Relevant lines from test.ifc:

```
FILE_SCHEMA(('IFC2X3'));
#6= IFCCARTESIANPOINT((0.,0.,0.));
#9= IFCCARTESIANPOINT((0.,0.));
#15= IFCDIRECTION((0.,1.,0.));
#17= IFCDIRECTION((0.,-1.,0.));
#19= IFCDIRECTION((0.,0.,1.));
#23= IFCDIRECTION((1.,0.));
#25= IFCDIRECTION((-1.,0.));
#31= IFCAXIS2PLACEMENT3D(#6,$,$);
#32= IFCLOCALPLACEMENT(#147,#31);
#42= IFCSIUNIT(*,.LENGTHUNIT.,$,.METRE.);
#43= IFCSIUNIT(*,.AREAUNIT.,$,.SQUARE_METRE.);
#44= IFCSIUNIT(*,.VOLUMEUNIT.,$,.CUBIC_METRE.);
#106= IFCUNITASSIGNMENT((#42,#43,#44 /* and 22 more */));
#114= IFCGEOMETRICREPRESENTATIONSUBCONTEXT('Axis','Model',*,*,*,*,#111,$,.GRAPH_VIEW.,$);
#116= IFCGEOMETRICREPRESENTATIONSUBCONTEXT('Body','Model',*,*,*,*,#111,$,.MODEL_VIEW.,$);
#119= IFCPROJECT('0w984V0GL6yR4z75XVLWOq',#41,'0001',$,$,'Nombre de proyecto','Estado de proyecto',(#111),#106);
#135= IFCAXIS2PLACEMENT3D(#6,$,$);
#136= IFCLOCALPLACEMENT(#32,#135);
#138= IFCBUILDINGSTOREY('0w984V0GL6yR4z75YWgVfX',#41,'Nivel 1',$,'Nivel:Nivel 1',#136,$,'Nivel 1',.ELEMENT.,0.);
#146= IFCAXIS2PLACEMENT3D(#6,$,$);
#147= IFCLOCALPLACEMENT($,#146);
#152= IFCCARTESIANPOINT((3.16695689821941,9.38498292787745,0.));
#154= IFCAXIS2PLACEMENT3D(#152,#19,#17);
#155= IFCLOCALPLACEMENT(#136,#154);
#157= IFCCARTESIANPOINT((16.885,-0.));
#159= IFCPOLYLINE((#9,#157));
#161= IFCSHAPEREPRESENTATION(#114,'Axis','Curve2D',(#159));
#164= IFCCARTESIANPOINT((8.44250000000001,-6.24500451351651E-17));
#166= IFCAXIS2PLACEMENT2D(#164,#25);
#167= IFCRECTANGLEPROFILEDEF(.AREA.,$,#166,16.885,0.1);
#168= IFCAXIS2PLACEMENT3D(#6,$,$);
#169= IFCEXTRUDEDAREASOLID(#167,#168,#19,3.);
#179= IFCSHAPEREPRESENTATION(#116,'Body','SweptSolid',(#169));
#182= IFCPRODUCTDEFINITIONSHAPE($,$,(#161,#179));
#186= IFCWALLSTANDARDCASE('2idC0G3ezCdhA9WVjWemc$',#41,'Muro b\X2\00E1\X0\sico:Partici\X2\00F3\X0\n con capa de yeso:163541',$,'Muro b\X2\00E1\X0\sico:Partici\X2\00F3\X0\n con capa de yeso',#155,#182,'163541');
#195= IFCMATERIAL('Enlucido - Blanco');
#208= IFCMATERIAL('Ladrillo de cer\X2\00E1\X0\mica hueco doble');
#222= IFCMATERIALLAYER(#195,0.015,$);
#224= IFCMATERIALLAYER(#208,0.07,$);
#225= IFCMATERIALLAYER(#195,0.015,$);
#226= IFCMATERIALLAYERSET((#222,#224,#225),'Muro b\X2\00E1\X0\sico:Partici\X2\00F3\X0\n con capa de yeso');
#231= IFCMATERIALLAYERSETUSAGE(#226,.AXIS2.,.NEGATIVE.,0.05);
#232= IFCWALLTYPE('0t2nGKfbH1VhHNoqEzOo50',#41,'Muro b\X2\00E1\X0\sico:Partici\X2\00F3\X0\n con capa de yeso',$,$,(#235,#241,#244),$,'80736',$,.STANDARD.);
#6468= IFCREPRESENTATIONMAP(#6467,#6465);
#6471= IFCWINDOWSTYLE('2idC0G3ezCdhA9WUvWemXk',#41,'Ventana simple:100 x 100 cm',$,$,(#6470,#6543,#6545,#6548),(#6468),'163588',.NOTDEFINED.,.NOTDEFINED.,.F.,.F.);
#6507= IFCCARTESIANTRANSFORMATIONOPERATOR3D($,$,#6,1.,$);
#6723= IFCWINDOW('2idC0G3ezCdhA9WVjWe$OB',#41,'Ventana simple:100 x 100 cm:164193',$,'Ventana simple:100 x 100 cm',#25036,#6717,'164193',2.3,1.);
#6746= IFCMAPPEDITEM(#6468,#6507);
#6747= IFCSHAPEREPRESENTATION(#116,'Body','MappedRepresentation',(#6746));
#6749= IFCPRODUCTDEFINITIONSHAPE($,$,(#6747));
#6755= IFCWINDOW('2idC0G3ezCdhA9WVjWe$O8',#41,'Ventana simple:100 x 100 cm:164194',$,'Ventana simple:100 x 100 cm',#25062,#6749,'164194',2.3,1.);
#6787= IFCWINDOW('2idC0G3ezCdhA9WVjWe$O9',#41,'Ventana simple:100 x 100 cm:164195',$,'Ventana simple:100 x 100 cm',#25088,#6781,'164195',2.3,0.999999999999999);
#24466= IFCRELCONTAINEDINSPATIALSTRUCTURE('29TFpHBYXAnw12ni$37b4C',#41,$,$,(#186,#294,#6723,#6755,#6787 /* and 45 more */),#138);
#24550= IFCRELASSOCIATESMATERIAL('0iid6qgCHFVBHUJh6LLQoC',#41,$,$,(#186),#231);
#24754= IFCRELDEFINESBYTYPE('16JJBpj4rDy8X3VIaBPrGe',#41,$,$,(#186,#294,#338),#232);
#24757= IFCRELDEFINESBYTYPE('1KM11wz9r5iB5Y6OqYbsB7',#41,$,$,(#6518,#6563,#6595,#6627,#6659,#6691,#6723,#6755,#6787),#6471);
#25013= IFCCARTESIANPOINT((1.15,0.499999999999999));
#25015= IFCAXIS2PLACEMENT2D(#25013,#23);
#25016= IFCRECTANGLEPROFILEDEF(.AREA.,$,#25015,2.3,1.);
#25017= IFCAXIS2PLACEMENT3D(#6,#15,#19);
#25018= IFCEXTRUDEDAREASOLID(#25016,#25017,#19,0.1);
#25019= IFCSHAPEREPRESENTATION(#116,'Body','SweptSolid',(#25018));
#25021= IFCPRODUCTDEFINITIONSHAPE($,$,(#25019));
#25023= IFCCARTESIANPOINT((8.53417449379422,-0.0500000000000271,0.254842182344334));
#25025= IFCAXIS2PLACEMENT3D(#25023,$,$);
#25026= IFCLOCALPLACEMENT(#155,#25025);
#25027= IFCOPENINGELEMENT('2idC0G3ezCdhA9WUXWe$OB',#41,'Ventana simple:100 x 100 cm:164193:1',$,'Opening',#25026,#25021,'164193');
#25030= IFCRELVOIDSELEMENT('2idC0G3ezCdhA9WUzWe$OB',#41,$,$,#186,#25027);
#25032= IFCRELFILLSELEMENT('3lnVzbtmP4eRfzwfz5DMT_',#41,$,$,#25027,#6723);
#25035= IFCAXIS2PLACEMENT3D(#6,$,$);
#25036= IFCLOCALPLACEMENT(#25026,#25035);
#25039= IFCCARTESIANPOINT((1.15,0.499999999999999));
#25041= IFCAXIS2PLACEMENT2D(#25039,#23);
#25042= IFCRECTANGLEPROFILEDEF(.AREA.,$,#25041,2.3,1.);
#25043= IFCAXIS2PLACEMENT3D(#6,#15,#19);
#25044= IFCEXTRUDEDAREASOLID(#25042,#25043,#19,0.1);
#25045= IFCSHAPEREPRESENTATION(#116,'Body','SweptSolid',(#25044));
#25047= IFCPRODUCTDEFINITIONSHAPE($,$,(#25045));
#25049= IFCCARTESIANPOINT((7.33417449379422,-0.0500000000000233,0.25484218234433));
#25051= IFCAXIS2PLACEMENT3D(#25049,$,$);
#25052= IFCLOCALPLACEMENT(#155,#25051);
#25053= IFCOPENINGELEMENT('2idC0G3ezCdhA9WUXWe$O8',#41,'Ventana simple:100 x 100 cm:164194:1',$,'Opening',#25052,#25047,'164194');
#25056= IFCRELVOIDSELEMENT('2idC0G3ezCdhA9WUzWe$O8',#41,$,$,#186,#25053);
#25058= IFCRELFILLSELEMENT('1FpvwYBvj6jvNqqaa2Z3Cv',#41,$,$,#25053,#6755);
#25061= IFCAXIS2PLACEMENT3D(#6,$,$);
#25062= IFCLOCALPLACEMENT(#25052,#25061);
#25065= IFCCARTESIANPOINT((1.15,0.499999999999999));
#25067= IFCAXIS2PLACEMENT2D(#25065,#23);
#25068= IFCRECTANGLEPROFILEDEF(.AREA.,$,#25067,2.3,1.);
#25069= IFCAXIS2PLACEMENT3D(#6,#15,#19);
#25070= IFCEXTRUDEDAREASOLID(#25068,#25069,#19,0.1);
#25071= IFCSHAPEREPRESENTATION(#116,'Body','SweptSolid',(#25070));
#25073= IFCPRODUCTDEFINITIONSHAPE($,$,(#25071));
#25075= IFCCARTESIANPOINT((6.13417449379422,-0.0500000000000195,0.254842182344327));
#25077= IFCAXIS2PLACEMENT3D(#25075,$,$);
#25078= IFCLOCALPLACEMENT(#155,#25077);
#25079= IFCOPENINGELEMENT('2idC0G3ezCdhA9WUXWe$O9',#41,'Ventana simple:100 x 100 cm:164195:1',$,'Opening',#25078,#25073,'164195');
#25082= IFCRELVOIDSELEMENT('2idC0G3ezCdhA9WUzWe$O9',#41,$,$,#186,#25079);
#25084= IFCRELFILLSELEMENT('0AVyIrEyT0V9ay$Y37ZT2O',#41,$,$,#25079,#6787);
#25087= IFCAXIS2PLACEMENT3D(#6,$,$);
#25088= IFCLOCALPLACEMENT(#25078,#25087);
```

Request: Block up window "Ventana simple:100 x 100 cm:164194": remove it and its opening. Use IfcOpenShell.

```python
import ifcopenshell
import ifcopenshell.api.feature
import ifcopenshell.api.root
import ifcopenshell.geom
import ifcopenshell.util.shape

model = ifcopenshell.open("test.ifc")
settings = ifcopenshell.geom.settings()


def volume(element):
    """Net volume in cubic metres, openings subtracted."""
    shape = ifcopenshell.geom.create_shape(settings, element)
    return ifcopenshell.util.shape.get_volume(shape.geometry)


window = model.by_id(6755)
opening = window.FillsVoids[0].RelatingOpeningElement
wall = opening.VoidsElements[0].RelatingBuildingElement
before = volume(wall)

ifcopenshell.api.root.remove_product(model, product=window)
ifcopenshell.api.feature.remove_feature(model, feature=opening)

after = volume(wall)

print(f"wall volume {before:.3f} -> {after:.3f} m3")

model.write("test_v2.ifc")
```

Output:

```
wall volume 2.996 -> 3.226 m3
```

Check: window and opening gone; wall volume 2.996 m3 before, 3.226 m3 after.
